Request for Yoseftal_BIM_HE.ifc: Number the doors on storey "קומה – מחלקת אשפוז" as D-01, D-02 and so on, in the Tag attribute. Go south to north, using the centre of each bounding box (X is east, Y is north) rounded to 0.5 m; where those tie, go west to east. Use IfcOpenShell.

First a look at what the model holds.

```python
import ifcopenshell
import ifcopenshell.util.element
import ifcopenshell.util.placement

model = ifcopenshell.open("Yoseftal_BIM_HE.ifc")
print(model.schema)
storey = next(s for s in model.by_type("IfcBuildingStorey") if s.Name == "קומה – מחלקת אשפוז")
doors = [e for e in ifcopenshell.util.element.get_decomposition(storey) if e.is_a("IfcDoor")]
for e in sorted(doors, key=lambda e: e.id()):
    origin = ifcopenshell.util.placement.get_local_placement(e.ObjectPlacement)[:3, 3]
    print(e.id(), e.Tag, e.Name, origin.round(2) + 0.0, sep=" | ")
```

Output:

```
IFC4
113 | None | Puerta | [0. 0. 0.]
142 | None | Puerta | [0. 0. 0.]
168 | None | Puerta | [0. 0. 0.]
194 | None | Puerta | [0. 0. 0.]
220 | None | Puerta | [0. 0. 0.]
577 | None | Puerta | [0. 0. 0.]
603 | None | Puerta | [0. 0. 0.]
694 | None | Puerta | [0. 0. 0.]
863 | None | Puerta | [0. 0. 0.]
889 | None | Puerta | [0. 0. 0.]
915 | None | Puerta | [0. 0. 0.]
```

```python
import ifcopenshell
import ifcopenshell.geom
import ifcopenshell.util.element
import ifcopenshell.util.shape

model = ifcopenshell.open("Yoseftal_BIM_HE.ifc")
settings = ifcopenshell.geom.settings()
settings.set("use-world-coords", True)


def centre(element):
    shape = ifcopenshell.geom.create_shape(settings, element)
    return ifcopenshell.util.shape.get_bbox_centroid(shape.geometry)


storey = next(s for s in model.by_type("IfcBuildingStorey") if s.Name == "קומה – מחלקת אשפוז")
doors = [e for e in ifcopenshell.util.element.get_decomposition(storey) if e.is_a("IfcDoor")]

# Insertion points can sit at a corner or the storey origin, so sort by the geometry (in metres).
centres = {e: centre(e) for e in doors}
doors.sort(key=lambda e: (round(centres[e][1] / 0.5), centres[e][0]))

for i, e in enumerate(doors, start=1):
    number = f"D-{i:02d}"
    e.Tag = number
    print(e.id(), number)

model.write("Yoseftal_BIM_HE-out.ifc")
```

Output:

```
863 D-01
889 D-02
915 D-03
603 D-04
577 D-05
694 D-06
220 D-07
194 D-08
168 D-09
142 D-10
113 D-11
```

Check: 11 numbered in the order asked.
